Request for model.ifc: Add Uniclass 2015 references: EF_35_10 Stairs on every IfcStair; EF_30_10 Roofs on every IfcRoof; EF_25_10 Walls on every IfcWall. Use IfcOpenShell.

First a look at what the model holds.

```python
import ifcopenshell

model = ifcopenshell.open("model.ifc")
print(model.schema)
print("classifications:", [c.Name for c in model.by_type("IfcClassification")])
for ifc_class in ("IfcDoor", "IfcRoof", "IfcStair", "IfcWall", "IfcWindow"):
    print(ifc_class, len(model.by_type(ifc_class)))
```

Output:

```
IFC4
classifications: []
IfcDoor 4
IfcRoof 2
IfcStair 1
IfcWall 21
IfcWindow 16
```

```python
import ifcopenshell
import ifcopenshell.api.classification

model = ifcopenshell.open("model.ifc")

system = ifcopenshell.api.classification.add_classification(model, classification="Uniclass 2015")

codes = {
    "IfcStair": ("EF_35_10", "Stairs"),
    "IfcRoof": ("EF_30_10", "Roofs"),
    "IfcWall": ("EF_25_10", "Walls"),
}
for ifc_class, (code, name) in codes.items():
    products = model.by_type(ifc_class)
    ifcopenshell.api.classification.add_reference(
        model, products=products, classification=system, identification=code, name=name
    )
    print(code, len(products))

model.write("model_updated.ifc")
```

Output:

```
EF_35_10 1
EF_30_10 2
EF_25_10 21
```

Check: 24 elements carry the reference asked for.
